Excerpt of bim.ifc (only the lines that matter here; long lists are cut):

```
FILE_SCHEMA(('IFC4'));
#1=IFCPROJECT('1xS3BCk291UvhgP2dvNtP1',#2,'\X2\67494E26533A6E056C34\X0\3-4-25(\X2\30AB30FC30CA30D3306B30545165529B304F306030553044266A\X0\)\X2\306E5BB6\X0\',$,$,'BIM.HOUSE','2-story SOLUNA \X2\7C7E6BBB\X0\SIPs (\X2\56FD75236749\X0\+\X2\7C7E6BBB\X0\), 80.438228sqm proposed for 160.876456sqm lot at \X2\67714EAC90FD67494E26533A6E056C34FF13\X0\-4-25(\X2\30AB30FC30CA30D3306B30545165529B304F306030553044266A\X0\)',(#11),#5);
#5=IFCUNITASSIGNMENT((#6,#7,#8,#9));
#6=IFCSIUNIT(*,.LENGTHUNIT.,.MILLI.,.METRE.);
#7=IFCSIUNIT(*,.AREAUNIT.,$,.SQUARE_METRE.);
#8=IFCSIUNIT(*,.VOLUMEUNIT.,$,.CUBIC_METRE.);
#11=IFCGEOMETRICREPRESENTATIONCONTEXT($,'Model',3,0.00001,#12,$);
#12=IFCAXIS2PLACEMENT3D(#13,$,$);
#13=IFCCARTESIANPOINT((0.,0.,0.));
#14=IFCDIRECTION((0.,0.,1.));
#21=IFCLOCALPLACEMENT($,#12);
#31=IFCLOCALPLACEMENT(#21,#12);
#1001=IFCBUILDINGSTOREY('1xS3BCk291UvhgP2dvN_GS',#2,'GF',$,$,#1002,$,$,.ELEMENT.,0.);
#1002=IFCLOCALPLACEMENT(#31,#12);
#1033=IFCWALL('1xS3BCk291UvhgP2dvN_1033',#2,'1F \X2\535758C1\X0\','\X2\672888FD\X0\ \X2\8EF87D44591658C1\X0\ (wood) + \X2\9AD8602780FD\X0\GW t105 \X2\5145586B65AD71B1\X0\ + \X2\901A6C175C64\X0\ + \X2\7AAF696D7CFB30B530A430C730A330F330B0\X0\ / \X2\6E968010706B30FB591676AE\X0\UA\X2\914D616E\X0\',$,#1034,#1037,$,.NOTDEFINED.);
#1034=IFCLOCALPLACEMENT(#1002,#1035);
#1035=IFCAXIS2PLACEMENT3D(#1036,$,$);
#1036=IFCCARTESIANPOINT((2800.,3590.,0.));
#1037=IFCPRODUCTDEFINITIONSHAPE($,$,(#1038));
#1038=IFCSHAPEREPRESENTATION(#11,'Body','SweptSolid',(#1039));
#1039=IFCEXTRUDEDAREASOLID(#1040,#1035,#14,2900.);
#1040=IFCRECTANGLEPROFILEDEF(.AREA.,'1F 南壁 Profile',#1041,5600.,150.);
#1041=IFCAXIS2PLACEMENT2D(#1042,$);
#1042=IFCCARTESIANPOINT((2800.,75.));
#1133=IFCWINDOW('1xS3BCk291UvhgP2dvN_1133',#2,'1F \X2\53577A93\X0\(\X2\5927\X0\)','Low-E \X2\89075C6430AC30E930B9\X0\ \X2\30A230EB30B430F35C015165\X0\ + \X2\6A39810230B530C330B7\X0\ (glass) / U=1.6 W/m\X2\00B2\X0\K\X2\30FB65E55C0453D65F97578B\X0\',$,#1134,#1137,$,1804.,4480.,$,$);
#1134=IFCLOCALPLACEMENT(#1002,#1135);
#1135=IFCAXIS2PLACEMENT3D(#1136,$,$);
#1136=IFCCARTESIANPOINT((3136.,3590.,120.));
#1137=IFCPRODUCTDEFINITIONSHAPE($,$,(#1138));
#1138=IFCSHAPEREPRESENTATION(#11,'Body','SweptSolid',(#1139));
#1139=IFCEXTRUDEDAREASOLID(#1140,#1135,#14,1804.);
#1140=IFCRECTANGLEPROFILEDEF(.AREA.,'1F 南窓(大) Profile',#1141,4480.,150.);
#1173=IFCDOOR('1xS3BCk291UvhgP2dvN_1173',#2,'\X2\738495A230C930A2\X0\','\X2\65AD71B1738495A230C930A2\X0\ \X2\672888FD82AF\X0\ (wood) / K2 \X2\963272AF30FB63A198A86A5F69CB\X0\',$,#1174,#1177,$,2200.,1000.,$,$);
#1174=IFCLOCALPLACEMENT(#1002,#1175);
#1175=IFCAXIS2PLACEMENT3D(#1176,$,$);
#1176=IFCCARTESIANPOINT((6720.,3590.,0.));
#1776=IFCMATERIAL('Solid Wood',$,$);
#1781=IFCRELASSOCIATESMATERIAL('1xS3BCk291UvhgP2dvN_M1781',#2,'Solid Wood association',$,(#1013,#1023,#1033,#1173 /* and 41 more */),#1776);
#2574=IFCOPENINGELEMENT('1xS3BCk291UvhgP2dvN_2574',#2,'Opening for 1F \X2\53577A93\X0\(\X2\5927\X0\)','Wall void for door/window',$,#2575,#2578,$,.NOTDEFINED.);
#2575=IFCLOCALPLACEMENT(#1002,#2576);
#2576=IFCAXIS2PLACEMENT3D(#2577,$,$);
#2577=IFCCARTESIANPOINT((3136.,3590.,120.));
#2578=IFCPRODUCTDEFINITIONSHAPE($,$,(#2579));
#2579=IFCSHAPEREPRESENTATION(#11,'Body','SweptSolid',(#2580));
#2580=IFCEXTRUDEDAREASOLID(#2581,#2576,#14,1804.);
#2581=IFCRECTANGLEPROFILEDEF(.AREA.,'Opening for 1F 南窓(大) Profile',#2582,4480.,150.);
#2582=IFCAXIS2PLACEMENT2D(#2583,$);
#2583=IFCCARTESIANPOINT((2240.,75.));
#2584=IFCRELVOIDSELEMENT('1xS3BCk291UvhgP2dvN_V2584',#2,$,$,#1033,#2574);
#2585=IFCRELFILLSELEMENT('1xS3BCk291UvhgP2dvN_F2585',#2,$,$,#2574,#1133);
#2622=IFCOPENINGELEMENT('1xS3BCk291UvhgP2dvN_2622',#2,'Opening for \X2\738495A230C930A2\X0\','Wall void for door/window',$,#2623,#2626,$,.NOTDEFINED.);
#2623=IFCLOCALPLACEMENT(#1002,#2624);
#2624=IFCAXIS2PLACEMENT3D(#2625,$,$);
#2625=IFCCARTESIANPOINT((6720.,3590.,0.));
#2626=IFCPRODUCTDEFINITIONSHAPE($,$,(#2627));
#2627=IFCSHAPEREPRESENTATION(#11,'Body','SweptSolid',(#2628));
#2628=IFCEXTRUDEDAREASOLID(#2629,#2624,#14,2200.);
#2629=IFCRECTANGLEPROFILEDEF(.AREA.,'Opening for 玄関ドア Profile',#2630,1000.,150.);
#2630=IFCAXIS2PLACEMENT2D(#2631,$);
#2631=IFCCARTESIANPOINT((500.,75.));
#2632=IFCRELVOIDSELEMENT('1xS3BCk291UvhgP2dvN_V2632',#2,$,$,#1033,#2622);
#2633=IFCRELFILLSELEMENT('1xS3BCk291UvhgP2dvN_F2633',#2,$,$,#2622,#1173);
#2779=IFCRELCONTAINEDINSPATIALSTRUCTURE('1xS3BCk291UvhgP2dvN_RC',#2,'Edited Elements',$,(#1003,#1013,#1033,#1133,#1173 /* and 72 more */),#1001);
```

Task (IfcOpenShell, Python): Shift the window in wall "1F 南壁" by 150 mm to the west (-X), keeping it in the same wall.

```python
import ifcopenshell
import ifcopenshell.api.geometry
import ifcopenshell.util.placement

model = ifcopenshell.open("bim.ifc")

window = model.by_guid("1xS3BCk291UvhgP2dvN_1133")
opening = window.FillsVoids[0].RelatingOpeningElement
wall = opening.VoidsElements[0].RelatingBuildingElement

wall_matrix = ifcopenshell.util.placement.get_local_placement(wall.ObjectPlacement)
shift = wall_matrix[:3, 0] * -150.0
before = ifcopenshell.util.placement.get_local_placement(window.ObjectPlacement)[:3, 3].copy()

# The window is not placed relative to its opening, so move both.
for product in (opening, window):
    matrix = ifcopenshell.util.placement.get_local_placement(product.ObjectPlacement)
    matrix[:3, 3] += shift
    ifcopenshell.api.geometry.edit_object_placement(model, product=product, matrix=matrix, is_si=False)

after = ifcopenshell.util.placement.get_local_placement(window.ObjectPlacement)[:3, 3]
print("window moved by", (after - before).round(3) + 0.0)

model.write("bim_rev.ifc")
```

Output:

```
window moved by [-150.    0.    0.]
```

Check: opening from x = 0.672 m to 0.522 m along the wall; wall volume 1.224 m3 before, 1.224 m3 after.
